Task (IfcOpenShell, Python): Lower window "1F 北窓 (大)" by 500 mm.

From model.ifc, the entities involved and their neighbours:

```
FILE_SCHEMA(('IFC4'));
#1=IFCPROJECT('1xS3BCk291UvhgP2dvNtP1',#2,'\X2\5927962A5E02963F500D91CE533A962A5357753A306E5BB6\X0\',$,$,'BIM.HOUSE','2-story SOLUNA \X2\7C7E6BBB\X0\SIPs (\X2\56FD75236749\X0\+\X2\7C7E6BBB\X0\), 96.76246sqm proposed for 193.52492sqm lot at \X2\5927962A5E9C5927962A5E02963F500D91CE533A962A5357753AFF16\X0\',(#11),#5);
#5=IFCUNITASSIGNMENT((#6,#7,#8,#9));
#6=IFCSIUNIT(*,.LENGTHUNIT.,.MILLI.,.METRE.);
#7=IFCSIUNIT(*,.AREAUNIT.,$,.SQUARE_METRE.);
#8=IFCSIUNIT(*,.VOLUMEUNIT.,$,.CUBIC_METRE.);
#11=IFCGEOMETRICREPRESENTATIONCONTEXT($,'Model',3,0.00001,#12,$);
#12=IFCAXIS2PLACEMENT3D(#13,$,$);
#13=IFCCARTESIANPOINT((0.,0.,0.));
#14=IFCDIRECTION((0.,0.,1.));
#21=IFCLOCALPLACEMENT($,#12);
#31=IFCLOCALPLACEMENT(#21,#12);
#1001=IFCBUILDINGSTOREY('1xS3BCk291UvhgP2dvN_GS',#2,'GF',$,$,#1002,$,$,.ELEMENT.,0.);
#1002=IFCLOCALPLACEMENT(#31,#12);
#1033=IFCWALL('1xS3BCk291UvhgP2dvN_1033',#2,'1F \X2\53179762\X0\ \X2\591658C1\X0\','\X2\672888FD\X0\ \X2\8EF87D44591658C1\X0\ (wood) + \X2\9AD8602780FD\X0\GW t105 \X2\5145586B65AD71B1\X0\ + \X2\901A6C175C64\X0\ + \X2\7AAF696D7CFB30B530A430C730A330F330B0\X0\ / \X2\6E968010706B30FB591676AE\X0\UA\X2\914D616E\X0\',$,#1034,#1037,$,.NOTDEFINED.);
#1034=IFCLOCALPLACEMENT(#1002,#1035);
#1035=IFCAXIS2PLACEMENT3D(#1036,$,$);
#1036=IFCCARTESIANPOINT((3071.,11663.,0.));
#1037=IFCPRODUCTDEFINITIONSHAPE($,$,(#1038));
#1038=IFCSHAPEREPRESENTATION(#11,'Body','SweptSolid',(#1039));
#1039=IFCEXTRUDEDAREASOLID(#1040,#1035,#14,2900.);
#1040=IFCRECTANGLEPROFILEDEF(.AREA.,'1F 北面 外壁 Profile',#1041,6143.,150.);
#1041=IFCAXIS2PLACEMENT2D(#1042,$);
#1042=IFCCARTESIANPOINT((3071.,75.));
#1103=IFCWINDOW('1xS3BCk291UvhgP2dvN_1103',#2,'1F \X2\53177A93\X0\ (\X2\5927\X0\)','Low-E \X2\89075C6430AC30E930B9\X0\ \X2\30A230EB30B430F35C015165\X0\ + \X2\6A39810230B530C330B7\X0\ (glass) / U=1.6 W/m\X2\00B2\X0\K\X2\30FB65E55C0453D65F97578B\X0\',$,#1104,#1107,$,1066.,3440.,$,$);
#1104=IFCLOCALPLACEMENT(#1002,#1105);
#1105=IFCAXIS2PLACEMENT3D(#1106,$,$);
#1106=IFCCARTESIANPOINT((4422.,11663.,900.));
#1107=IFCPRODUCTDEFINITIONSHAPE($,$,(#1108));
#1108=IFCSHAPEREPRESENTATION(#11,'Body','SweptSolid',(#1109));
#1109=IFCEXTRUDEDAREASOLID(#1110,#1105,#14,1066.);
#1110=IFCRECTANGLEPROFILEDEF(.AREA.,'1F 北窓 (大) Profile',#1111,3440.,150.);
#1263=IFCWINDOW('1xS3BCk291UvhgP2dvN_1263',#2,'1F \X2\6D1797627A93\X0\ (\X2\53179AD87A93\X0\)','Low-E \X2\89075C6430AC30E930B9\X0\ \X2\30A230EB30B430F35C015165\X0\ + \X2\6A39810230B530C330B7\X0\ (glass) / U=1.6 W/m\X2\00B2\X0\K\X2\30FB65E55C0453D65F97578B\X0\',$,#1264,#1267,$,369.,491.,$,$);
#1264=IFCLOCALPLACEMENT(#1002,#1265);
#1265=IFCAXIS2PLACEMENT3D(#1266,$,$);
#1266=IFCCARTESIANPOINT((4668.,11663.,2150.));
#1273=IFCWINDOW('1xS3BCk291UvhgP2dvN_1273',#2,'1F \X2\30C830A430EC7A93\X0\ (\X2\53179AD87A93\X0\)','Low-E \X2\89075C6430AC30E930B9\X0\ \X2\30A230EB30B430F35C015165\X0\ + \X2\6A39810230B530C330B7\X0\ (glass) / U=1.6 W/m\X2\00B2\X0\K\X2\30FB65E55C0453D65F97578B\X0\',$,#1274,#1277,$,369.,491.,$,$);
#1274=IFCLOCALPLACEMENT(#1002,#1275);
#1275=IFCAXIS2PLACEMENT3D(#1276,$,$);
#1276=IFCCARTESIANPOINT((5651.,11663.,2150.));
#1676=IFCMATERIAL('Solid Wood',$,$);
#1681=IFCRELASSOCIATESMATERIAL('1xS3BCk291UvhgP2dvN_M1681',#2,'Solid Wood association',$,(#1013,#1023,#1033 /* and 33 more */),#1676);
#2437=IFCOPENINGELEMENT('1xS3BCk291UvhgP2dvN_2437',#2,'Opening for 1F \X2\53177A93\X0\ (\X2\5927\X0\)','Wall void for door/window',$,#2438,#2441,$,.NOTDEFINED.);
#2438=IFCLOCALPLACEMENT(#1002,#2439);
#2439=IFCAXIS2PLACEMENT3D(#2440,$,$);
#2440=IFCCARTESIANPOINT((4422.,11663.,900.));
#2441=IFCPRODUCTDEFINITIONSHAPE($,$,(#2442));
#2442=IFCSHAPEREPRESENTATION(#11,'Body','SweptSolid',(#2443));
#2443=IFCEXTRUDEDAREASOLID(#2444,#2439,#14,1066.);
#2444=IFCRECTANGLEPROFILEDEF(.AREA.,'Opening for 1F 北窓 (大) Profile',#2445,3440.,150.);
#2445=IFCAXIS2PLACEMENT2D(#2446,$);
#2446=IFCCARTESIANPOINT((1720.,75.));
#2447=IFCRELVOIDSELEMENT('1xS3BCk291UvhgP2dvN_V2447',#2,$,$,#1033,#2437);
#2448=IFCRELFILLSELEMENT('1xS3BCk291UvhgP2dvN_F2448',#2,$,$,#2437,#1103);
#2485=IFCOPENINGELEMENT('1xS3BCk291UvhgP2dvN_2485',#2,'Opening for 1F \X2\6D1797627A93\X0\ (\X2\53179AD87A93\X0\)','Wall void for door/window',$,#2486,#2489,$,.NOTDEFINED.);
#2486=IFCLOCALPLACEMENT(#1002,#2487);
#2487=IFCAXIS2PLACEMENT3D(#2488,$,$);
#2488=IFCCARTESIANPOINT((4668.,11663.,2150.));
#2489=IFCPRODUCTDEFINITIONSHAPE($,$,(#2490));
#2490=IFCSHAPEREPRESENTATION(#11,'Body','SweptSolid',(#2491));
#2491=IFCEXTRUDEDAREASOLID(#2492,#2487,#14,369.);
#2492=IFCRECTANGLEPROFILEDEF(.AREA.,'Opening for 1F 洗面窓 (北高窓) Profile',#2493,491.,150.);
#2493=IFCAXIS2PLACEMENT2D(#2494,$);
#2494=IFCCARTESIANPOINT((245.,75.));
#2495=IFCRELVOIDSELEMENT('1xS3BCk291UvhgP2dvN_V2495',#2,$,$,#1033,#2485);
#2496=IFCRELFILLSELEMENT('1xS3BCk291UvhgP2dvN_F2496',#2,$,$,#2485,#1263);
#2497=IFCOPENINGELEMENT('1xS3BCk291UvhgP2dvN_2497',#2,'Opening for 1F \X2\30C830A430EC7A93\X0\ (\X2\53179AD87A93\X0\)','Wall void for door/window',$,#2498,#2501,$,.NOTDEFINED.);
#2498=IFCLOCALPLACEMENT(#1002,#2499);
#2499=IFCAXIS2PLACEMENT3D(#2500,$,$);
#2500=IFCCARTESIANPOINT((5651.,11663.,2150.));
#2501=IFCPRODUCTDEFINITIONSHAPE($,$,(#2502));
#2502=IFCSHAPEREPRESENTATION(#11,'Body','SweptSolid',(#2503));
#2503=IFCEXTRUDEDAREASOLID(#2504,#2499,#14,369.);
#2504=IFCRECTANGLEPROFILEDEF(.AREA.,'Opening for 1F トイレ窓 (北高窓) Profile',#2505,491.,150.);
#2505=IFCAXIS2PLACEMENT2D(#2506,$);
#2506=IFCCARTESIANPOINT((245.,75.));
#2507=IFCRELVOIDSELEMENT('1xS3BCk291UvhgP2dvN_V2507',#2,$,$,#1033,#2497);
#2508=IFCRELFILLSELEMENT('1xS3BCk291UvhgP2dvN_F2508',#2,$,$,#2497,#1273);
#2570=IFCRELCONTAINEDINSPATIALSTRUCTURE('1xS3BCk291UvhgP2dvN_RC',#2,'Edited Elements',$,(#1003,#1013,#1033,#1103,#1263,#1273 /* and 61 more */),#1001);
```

```python
import numpy as np
import ifcopenshell
import ifcopenshell.api.geometry
import ifcopenshell.util.placement
import ifcopenshell.util.unit

model = ifcopenshell.open("model.ifc")
unit_scale = ifcopenshell.util.unit.calculate_unit_scale(model)

window = model.by_guid("1xS3BCk291UvhgP2dvN_1103")
opening = window.FillsVoids[0].RelatingOpeningElement
dz = -0.5 / unit_scale

shift = np.array([0.0, 0.0, dz])
# The window is not placed relative to its opening, so move both.
for product in (opening, window):
    matrix = ifcopenshell.util.placement.get_local_placement(product.ObjectPlacement)
    matrix[:3, 3] += shift
    ifcopenshell.api.geometry.edit_object_placement(model, product=product, matrix=matrix, is_si=False)

print(f"moved by {dz * unit_scale:+.3f} m")

model.write("model_v2.ifc")
```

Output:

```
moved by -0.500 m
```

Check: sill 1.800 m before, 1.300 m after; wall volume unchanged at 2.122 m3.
